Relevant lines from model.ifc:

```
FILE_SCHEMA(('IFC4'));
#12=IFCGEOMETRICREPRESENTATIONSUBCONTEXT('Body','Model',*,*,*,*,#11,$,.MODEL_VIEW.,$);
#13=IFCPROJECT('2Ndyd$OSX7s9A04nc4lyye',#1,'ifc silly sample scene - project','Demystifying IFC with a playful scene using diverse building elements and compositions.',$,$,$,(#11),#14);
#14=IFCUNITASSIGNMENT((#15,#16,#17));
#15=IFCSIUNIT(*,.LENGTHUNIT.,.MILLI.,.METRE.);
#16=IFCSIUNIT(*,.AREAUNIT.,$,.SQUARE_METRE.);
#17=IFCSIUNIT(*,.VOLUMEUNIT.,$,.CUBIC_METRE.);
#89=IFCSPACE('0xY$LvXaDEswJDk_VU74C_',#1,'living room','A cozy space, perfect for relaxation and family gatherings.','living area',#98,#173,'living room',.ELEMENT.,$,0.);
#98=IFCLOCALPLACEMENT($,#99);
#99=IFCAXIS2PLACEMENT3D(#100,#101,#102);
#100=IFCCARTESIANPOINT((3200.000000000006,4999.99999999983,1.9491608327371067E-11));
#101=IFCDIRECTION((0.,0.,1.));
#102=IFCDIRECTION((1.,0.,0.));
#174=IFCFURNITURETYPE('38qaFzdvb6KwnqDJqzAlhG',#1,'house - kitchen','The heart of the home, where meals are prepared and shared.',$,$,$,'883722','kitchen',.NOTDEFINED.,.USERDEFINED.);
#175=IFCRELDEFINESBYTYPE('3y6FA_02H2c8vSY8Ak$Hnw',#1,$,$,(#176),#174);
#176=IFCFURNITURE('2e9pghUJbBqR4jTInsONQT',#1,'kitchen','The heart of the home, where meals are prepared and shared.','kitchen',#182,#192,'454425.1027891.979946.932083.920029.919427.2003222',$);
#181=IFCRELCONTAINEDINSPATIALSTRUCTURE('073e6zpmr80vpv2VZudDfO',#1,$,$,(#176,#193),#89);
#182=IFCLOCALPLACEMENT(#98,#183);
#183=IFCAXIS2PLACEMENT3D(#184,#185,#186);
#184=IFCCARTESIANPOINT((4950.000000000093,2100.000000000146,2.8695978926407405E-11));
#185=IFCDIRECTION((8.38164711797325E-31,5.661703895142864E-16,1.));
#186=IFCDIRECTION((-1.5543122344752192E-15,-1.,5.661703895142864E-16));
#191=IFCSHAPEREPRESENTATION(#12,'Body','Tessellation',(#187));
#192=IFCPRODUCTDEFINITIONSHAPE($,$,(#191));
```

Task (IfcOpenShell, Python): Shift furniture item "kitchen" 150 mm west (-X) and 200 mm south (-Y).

```python
import ifcopenshell
import ifcopenshell.api.geometry
import ifcopenshell.util.placement

model = ifcopenshell.open("model.ifc")

item = model.by_id(176)
matrix = ifcopenshell.util.placement.get_local_placement(item.ObjectPlacement)
matrix[0, 3] -= 150.0
matrix[1, 3] -= 200.0
ifcopenshell.api.geometry.edit_object_placement(model, product=item, matrix=matrix, is_si=False)

print(ifcopenshell.util.placement.get_local_placement(item.ObjectPlacement).round(3) + 0.0)

model.write("model_edited.ifc")
```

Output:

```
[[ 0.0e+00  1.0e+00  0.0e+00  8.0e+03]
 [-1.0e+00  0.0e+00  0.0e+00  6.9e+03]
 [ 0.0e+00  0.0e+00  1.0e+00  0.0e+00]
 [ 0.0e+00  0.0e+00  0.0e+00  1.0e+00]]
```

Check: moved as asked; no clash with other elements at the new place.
